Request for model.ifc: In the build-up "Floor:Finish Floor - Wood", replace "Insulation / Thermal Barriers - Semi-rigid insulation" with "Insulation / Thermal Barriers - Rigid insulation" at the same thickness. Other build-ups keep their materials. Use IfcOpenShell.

First a look at what the model holds.

```python
import ifcopenshell
import ifcopenshell.util.element

model = ifcopenshell.open("model.ifc")
print(model.schema)
for layer_set in model.by_type("IfcMaterialLayerSet"):
    if layer_set.LayerSetName == "Floor:Finish Floor - Wood":
        for layer in layer_set.MaterialLayers:
            print(layer.id(), layer.Material and layer.Material.Name, layer.LayerThickness, sep=" | ")
        print(len(ifcopenshell.util.element.get_elements_by_material(model, layer_set)), "elements and types use it")
print(sorted(m.Name for m in model.by_type("IfcMaterial") if m.Name)[:60])
```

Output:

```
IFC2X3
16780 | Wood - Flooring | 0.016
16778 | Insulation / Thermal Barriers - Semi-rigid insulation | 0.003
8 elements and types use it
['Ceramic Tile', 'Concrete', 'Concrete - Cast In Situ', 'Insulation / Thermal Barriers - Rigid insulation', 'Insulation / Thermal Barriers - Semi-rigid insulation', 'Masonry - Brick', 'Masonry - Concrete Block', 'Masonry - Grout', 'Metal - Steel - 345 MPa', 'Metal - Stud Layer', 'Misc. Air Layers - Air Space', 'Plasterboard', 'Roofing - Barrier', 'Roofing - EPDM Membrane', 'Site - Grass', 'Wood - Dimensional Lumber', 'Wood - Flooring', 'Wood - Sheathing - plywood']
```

```python
import ifcopenshell
import ifcopenshell.api.material

model = ifcopenshell.open("model.ifc")

layer_set = next(s for s in model.by_type("IfcMaterialLayerSet") if s.LayerSetName == "Floor:Finish Floor - Wood")
layer = next(l for l in layer_set.MaterialLayers if l.Material and l.Material.Name == "Insulation / Thermal Barriers - Semi-rigid insulation")
material = next(m for m in model.by_type("IfcMaterial") if m.Name == "Insulation / Thermal Barriers - Rigid insulation")

# Point this one layer at the other material; renaming the old one would change it everywhere.
ifcopenshell.api.material.edit_layer(model, layer=layer, attributes={}, material=material)

print([l.Material.Name if l.Material else None for l in layer_set.MaterialLayers])

model.write("model_edited.ifc")
```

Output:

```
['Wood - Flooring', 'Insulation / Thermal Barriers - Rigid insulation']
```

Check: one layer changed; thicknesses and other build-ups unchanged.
